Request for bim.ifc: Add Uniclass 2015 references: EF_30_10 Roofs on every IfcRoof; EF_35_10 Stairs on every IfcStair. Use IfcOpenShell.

First a look at what the model holds.

```python
import ifcopenshell

model = ifcopenshell.open("bim.ifc")
print(model.schema)
print("classifications:", [c.Name for c in model.by_type("IfcClassification")])
for ifc_class in ("IfcDoor", "IfcRoof", "IfcStair", "IfcWall", "IfcWindow"):
    print(ifc_class, len(model.by_type(ifc_class)))
```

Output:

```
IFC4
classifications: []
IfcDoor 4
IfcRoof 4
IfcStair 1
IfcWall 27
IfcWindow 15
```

```python
import ifcopenshell
import ifcopenshell.api.classification

model = ifcopenshell.open("bim.ifc")

system = ifcopenshell.api.classification.add_classification(model, classification="Uniclass 2015")

codes = {
    "IfcRoof": ("EF_30_10", "Roofs"),
    "IfcStair": ("EF_35_10", "Stairs"),
}
for ifc_class, (code, name) in codes.items():
    products = model.by_type(ifc_class)
    ifcopenshell.api.classification.add_reference(
        model, products=products, classification=system, identification=code, name=name
    )
    print(code, len(products))

model.write("bim_rev.ifc")
```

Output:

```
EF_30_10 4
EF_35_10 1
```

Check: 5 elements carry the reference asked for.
